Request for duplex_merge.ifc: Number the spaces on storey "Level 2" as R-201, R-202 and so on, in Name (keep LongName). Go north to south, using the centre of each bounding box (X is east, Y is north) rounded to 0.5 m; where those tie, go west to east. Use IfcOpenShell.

First a look at what the model holds.

```python
import ifcopenshell
import ifcopenshell.util.element
import ifcopenshell.util.placement

model = ifcopenshell.open("duplex_merge.ifc")
print(model.schema)
storey = next(s for s in model.by_type("IfcBuildingStorey") if s.Name == "Level 2")
spaces = [e for e in ifcopenshell.util.element.get_decomposition(storey) if e.is_a("IfcSpace")]
for e in sorted(spaces, key=lambda e: e.id()):
    origin = ifcopenshell.util.placement.get_local_placement(e.ObjectPlacement)[:3, 3]
    print(e.id(), e.Name, e.LongName, origin.round(2) + 0.0, sep=" | ")
```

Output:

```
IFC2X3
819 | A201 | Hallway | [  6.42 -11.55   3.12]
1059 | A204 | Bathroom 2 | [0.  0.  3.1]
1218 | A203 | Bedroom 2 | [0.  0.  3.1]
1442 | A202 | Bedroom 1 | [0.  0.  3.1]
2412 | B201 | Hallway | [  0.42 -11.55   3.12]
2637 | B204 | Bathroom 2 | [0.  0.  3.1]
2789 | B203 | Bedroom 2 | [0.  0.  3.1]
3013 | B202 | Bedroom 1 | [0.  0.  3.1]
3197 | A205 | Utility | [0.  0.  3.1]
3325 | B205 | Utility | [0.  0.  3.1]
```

```python
import ifcopenshell
import ifcopenshell.geom
import ifcopenshell.util.element
import ifcopenshell.util.shape

model = ifcopenshell.open("duplex_merge.ifc")
settings = ifcopenshell.geom.settings()
settings.set("use-world-coords", True)


def centre(element):
    shape = ifcopenshell.geom.create_shape(settings, element)
    return ifcopenshell.util.shape.get_bbox_centroid(shape.geometry)


storey = next(s for s in model.by_type("IfcBuildingStorey") if s.Name == "Level 2")
spaces = [e for e in ifcopenshell.util.element.get_decomposition(storey) if e.is_a("IfcSpace")]

# Insertion points can sit at a corner or the storey origin, so sort by the geometry (in metres).
centres = {e: centre(e) for e in spaces}
spaces.sort(key=lambda e: (-round(centres[e][1] / 0.5), centres[e][0]))

for i, e in enumerate(spaces, start=1):
    number = f"R-2{i:02d}"
    e.Name = number
    print(e.id(), number)

model.write("duplex_merge_v2.ifc")
```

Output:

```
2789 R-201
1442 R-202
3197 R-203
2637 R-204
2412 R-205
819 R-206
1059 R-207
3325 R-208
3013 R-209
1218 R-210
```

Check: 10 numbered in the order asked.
